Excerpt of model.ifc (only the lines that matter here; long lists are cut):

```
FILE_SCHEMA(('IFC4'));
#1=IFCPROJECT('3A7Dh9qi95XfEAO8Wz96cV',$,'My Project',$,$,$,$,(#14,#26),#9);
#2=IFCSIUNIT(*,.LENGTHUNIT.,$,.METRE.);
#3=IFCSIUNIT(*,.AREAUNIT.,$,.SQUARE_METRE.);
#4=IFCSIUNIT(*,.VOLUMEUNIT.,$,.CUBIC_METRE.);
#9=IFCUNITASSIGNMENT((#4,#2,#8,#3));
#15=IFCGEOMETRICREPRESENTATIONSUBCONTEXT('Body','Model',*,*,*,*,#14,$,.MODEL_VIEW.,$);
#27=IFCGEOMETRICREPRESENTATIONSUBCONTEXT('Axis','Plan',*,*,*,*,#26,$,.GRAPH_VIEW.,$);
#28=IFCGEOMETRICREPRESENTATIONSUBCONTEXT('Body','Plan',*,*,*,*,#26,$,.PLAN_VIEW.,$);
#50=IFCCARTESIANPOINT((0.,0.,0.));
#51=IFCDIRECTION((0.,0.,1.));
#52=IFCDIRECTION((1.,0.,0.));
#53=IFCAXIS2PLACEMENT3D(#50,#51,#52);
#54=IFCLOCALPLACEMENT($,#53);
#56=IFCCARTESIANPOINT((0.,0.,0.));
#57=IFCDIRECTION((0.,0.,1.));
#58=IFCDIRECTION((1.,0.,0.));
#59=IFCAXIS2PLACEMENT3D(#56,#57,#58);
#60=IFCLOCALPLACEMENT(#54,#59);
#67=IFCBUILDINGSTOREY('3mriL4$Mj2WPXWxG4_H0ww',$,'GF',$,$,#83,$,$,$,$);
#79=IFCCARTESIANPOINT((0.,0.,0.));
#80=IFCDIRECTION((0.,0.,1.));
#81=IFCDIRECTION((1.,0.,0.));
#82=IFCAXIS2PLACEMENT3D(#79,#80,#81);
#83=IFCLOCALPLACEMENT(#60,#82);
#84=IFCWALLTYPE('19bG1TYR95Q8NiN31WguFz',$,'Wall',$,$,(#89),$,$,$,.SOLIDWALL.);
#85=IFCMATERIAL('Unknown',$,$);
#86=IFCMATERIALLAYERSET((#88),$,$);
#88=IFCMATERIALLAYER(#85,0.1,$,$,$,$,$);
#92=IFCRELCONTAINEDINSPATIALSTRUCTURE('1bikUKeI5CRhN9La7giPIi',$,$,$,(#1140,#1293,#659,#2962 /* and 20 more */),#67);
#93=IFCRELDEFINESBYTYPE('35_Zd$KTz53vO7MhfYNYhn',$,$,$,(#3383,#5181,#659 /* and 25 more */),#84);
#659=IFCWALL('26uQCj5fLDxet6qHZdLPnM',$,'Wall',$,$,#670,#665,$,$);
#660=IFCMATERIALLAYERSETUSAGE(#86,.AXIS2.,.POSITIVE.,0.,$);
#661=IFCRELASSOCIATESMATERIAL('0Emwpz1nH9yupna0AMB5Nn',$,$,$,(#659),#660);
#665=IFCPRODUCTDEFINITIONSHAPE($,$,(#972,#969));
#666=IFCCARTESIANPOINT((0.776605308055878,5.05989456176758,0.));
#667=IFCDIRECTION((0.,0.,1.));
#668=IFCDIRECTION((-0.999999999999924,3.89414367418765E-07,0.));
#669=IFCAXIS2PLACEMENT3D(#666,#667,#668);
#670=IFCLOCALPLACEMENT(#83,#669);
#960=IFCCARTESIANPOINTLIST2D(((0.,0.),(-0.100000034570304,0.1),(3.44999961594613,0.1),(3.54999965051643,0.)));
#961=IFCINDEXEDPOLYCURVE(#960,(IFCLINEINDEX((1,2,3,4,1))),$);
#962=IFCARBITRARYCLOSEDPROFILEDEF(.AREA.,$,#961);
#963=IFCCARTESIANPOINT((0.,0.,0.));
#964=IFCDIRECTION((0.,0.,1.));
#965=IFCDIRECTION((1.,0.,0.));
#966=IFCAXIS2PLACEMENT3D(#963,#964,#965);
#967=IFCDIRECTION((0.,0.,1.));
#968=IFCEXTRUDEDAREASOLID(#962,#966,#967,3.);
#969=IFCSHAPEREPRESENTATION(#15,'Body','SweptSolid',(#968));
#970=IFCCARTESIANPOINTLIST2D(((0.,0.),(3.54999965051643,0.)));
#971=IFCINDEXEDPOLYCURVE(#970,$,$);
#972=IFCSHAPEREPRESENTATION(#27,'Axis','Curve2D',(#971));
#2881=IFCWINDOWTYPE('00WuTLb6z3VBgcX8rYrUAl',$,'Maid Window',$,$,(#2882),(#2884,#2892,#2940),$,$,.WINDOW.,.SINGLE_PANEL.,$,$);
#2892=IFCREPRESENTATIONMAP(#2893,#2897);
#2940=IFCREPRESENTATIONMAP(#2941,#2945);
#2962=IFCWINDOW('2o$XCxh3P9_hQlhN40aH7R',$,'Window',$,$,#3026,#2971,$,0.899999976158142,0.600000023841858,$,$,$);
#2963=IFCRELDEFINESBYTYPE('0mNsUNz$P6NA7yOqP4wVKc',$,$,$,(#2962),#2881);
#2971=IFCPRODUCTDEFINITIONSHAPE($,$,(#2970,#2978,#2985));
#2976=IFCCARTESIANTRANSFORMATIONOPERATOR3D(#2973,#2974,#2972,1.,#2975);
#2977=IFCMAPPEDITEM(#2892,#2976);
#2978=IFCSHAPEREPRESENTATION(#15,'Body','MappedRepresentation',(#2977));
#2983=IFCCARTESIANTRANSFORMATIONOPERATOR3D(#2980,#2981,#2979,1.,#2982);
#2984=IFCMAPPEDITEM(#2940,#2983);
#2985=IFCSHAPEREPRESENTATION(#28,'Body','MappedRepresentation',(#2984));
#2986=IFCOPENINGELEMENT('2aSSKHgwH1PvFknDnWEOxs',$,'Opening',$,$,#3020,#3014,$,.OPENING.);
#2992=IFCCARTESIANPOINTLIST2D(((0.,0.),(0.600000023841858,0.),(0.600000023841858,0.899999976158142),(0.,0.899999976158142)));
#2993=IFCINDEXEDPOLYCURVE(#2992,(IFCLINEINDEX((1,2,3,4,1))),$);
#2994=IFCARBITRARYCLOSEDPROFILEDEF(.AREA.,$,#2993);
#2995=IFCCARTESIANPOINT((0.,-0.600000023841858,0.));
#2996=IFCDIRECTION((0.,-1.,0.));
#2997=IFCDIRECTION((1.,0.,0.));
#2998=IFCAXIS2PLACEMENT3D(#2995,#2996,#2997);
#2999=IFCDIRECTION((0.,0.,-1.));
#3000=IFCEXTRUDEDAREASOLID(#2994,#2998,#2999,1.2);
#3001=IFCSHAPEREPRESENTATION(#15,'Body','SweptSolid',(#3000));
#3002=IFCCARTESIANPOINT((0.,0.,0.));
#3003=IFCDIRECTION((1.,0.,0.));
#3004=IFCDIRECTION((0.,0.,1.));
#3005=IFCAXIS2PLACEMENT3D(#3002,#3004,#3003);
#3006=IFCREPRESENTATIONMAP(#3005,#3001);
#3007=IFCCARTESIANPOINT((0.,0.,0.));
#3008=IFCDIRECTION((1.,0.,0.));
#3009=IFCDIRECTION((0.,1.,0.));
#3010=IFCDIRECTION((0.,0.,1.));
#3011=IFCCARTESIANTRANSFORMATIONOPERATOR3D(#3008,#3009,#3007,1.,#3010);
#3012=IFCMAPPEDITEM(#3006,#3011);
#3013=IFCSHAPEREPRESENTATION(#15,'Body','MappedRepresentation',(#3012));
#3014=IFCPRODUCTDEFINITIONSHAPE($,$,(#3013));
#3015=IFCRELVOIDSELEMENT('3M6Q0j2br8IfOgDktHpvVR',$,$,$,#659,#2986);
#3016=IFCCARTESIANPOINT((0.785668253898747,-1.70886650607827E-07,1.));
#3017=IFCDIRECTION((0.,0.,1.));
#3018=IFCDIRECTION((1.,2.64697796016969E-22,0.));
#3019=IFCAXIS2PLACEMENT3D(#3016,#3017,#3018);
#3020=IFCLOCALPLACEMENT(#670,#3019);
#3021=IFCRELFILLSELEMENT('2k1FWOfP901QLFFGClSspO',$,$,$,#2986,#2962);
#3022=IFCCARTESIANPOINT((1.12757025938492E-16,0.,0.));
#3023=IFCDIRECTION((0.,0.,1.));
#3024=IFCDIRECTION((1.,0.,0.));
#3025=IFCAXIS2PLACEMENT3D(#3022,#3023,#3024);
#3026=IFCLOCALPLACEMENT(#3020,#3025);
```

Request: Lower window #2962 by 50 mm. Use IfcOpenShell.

```python
import numpy as np
import ifcopenshell
import ifcopenshell.api.geometry
import ifcopenshell.util.placement
import ifcopenshell.util.unit

model = ifcopenshell.open("model.ifc")
unit_scale = ifcopenshell.util.unit.calculate_unit_scale(model)

window = model.by_guid("2o$XCxh3P9_hQlhN40aH7R")
opening = window.FillsVoids[0].RelatingOpeningElement
dz = -0.05 / unit_scale

shift = np.array([0.0, 0.0, dz])
# The window is placed relative to its opening, so it follows when the opening moves.
matrix = ifcopenshell.util.placement.get_local_placement(opening.ObjectPlacement)
matrix[:3, 3] += shift
ifcopenshell.api.geometry.edit_object_placement(
    model, product=opening, matrix=matrix, is_si=False, should_transform_children=True
)

print(f"moved by {dz * unit_scale:+.3f} m")

model.write("model-out.ifc")
```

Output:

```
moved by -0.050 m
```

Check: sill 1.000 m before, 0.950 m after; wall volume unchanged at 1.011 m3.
